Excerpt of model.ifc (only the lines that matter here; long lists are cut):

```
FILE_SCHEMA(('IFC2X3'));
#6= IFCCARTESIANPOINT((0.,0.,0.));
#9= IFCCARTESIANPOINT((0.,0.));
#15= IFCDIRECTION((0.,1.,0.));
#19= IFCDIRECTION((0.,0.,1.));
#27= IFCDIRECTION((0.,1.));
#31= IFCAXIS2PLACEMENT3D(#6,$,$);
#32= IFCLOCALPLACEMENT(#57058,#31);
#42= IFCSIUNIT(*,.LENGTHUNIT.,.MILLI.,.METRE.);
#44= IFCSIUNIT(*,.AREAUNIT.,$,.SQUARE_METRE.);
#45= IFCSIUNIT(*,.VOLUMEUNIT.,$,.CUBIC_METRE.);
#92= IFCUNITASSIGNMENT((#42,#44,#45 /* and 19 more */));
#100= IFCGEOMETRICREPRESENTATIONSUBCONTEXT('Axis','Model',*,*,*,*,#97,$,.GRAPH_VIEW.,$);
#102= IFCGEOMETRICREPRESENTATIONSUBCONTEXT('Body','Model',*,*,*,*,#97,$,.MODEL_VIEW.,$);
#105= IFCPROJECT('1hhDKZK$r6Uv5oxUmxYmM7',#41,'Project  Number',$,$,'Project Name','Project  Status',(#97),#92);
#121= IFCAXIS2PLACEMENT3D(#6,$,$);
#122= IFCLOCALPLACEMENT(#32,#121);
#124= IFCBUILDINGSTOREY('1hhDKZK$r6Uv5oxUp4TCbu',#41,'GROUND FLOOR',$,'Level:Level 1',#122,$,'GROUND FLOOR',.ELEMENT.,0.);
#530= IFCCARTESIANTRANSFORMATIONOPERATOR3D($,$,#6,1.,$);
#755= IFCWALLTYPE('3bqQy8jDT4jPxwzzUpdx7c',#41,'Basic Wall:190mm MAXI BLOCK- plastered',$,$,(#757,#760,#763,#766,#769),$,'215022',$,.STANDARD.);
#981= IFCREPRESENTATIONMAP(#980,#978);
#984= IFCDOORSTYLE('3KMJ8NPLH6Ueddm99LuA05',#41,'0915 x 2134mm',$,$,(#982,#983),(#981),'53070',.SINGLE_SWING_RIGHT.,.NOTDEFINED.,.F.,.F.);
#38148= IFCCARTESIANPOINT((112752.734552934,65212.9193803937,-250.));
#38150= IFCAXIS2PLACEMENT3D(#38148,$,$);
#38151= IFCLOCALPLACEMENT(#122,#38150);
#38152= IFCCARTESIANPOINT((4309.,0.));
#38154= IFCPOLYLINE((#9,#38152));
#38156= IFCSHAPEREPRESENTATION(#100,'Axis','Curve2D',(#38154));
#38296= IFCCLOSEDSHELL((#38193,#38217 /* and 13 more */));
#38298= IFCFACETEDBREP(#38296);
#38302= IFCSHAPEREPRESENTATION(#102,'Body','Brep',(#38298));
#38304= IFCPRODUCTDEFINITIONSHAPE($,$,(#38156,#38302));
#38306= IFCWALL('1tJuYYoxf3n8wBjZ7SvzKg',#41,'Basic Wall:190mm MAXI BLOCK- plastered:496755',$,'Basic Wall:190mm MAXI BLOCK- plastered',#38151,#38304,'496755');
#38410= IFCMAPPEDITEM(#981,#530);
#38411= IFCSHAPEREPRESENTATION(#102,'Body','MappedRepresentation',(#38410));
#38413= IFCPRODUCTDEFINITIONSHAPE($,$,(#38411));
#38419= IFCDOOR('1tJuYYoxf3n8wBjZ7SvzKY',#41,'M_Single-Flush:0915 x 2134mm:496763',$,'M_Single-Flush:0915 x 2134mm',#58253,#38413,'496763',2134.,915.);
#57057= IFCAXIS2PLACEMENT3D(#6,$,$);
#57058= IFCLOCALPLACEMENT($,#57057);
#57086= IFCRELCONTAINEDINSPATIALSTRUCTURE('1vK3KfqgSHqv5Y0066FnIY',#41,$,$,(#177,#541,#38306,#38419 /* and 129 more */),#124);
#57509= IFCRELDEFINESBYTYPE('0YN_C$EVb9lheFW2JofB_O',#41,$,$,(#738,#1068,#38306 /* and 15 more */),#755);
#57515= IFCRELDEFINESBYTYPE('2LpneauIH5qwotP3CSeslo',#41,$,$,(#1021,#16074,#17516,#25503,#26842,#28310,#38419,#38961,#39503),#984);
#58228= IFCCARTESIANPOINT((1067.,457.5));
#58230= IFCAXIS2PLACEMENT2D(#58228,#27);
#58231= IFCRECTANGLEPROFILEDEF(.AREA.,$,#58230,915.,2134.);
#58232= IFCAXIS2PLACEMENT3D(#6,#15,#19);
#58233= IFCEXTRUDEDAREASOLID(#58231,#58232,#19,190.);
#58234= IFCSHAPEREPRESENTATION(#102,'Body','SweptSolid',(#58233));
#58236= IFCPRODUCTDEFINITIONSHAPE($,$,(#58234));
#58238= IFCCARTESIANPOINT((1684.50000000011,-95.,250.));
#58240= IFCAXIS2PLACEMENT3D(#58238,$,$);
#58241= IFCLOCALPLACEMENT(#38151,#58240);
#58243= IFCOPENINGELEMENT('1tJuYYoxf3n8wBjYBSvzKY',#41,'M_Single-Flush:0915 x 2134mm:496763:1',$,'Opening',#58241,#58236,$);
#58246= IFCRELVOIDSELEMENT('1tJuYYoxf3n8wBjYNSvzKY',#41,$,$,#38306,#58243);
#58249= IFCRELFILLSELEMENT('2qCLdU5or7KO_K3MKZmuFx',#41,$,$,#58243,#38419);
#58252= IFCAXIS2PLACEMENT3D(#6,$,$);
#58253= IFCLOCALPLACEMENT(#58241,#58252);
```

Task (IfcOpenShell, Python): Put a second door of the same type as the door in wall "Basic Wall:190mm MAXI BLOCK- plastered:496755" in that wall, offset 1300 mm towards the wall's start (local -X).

```python
import ifcopenshell
import ifcopenshell.api.feature
import ifcopenshell.api.geometry
import ifcopenshell.api.root
import ifcopenshell.geom
import ifcopenshell.util.element
import ifcopenshell.util.placement
import ifcopenshell.util.shape

model = ifcopenshell.open("model.ifc")
settings = ifcopenshell.geom.settings()


def volume(element):
    """Net volume in cubic metres, openings subtracted."""
    shape = ifcopenshell.geom.create_shape(settings, element)
    return ifcopenshell.util.shape.get_volume(shape.geometry)


def reuse_history(source, copy):
    """copy_class also copies each property set's owner history, people and application; keep the originals."""
    for rel in copy.IsDefinedBy:
        if rel.is_a("IfcRelDefinesByProperties") and (history := rel.RelatingPropertyDefinition.OwnerHistory):
            rel.RelatingPropertyDefinition.OwnerHistory = source.OwnerHistory
            ifcopenshell.util.element.remove_deep2(model, history)


door = model.by_guid("1tJuYYoxf3n8wBjZ7SvzKY")
opening = door.FillsVoids[0].RelatingOpeningElement
wall = opening.VoidsElements[0].RelatingBuildingElement
before = volume(wall)
shift = ifcopenshell.util.placement.get_local_placement(wall.ObjectPlacement)[:3, 0] * -1300.0

# copy_class copies the void relationship, type, container and properties, but no geometry.
new_opening = ifcopenshell.api.root.copy_class(model, product=opening)
new_opening.Representation = ifcopenshell.util.element.copy_deep(
    model, opening.Representation, exclude=["IfcGeometricRepresentationContext", "IfcRepresentationMap"]
)
new_opening.Name = "M_Single-Flush:0915 x 2134mm"
new_door = ifcopenshell.api.root.copy_class(model, product=door)
new_door.Representation = ifcopenshell.util.element.copy_deep(
    model, door.Representation, exclude=["IfcGeometricRepresentationContext", "IfcRepresentationMap"]
)
new_door.Name = "M_Single-Flush:0915 x 2134mm"
new_door.Tag = None
reuse_history(door, new_door)
fills = ifcopenshell.api.feature.add_filling(model, opening=new_opening, element=new_door)
fills.OwnerHistory = new_door.OwnerHistory  # required in IFC2X3

for old, new in ((opening, new_opening), (door, new_door)):
    matrix = ifcopenshell.util.placement.get_local_placement(old.ObjectPlacement)
    matrix[:3, 3] += shift
    ifcopenshell.api.geometry.edit_object_placement(model, product=new, matrix=matrix, is_si=False)

after = volume(wall)

print(f"wall volume {before:.3f} -> {after:.3f} m3")

model.write("model_v2.ifc")
```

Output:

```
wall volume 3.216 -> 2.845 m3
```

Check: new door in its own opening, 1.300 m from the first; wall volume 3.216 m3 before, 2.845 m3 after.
